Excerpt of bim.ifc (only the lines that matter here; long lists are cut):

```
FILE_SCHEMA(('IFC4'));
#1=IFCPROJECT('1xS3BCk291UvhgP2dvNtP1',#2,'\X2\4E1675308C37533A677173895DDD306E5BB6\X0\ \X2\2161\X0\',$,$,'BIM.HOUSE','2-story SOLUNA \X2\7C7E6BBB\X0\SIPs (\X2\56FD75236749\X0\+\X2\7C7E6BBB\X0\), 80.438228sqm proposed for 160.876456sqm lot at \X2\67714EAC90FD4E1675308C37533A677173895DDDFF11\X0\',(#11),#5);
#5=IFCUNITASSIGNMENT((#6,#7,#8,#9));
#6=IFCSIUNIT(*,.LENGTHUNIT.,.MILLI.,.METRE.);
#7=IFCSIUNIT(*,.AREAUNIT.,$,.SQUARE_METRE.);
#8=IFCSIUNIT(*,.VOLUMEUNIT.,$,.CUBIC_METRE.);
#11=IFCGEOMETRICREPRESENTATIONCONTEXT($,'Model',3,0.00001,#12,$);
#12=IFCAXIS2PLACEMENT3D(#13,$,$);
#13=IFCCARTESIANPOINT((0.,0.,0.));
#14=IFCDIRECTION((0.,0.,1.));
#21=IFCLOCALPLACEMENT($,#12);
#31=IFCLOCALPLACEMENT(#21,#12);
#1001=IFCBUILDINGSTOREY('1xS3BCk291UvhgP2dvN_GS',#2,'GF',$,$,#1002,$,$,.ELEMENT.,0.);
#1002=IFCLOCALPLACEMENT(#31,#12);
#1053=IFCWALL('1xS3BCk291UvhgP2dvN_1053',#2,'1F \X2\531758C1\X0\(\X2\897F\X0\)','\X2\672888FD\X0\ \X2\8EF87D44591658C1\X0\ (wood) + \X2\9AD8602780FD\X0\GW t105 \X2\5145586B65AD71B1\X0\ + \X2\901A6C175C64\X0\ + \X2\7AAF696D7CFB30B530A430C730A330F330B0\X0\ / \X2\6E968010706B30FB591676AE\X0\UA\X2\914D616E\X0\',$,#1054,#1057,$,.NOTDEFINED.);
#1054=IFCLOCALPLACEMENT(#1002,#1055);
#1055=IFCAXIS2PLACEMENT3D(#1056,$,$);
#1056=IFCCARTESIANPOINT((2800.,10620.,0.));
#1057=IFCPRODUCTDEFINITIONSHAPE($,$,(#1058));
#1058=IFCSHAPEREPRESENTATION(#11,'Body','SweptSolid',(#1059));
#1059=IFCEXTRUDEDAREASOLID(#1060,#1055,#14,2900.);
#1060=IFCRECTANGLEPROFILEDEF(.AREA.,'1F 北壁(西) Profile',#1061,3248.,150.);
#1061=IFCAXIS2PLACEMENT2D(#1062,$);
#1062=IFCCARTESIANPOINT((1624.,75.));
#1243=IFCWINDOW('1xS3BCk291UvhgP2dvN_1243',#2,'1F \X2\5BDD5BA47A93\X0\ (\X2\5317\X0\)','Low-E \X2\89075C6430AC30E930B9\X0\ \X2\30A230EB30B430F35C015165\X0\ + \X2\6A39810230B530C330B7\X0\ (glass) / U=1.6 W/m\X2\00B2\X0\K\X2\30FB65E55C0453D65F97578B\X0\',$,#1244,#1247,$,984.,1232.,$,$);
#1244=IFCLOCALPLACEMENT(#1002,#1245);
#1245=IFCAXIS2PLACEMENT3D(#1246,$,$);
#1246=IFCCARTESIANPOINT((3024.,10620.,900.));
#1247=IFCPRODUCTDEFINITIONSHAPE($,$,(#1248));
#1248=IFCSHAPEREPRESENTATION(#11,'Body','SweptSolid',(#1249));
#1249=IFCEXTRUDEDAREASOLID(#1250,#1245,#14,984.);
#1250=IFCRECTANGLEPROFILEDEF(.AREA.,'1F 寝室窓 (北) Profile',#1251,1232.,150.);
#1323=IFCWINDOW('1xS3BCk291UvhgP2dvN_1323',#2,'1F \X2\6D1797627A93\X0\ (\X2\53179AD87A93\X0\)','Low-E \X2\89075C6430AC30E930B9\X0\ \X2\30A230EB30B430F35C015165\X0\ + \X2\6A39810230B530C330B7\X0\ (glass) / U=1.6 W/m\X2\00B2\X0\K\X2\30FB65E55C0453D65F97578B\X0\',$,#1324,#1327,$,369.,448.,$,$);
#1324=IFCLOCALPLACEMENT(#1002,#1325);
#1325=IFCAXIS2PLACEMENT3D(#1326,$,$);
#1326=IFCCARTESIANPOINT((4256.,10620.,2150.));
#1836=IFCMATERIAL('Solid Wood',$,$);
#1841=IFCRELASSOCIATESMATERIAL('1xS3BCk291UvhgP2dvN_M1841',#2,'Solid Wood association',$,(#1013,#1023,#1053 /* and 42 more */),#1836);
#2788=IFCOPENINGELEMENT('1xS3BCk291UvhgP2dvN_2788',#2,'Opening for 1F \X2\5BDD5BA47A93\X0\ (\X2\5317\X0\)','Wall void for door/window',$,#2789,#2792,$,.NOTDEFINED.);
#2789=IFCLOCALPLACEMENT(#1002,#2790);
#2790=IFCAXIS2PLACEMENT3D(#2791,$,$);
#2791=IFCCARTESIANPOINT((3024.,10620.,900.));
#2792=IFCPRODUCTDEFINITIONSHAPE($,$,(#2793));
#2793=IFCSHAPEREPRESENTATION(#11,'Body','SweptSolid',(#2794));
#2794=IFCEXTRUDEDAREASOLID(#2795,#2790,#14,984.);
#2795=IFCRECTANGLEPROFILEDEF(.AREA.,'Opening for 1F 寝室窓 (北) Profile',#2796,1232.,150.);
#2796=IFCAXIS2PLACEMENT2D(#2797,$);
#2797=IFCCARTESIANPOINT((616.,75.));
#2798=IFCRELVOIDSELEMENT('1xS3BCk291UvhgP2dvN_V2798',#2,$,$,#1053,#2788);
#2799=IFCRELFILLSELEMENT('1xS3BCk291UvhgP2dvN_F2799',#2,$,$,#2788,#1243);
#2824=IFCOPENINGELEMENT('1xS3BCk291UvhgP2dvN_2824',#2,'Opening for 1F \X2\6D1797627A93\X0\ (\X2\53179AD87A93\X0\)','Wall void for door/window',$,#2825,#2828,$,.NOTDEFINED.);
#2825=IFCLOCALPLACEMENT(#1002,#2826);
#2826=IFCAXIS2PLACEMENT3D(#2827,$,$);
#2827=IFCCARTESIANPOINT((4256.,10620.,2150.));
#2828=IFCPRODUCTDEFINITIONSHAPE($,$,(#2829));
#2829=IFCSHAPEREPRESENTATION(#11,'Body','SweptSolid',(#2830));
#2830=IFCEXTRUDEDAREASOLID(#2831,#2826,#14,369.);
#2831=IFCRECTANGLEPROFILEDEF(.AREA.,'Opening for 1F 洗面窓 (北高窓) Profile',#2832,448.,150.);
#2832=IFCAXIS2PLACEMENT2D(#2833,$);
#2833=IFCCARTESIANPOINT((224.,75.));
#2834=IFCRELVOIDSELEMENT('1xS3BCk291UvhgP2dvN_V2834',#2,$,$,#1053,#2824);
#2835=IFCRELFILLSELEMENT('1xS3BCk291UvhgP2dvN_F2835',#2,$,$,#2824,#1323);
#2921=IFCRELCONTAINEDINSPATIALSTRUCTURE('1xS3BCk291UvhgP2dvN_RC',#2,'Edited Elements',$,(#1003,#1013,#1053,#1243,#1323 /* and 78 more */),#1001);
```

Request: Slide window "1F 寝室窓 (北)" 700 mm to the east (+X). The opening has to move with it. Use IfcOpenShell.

```python
import ifcopenshell
import ifcopenshell.api.geometry
import ifcopenshell.util.placement

model = ifcopenshell.open("bim.ifc")

window = model.by_id(1243)
opening = window.FillsVoids[0].RelatingOpeningElement
wall = opening.VoidsElements[0].RelatingBuildingElement

wall_matrix = ifcopenshell.util.placement.get_local_placement(wall.ObjectPlacement)
shift = wall_matrix[:3, 0] * 700.0
before = ifcopenshell.util.placement.get_local_placement(window.ObjectPlacement)[:3, 3].copy()

# The window is not placed relative to its opening, so move both.
for product in (opening, window):
    matrix = ifcopenshell.util.placement.get_local_placement(product.ObjectPlacement)
    matrix[:3, 3] += shift
    ifcopenshell.api.geometry.edit_object_placement(model, product=product, matrix=matrix, is_si=False)

after = ifcopenshell.util.placement.get_local_placement(window.ObjectPlacement)[:3, 3]
print("window moved by", (after - before).round(3) + 0.0)

model.write("bim-out.ifc")
```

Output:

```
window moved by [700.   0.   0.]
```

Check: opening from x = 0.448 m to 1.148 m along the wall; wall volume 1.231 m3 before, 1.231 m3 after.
